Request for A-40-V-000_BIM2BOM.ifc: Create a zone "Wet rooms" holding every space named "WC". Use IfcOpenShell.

First a look at what the model holds.

```python
import ifcopenshell

model = ifcopenshell.open("A-40-V-000_BIM2BOM.ifc")
print(model.schema)
seen = {}
for space in model.by_type("IfcSpace"):
    seen[space.LongName] = seen.get(space.LongName, 0) + 1
for name, count in sorted(seen.items(), key=str):
    print(count, "x", name)
print("zones:", [z.Name for z in model.by_type("IfcZone")][:20])
```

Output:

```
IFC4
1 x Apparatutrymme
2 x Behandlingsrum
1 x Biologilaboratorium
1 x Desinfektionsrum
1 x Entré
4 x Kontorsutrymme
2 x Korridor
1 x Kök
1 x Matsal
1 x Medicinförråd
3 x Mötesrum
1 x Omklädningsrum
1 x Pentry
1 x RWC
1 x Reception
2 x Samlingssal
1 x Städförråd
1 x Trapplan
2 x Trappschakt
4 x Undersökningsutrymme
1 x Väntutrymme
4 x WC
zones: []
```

```python
import ifcopenshell
import ifcopenshell.api.group
import ifcopenshell.api.root

model = ifcopenshell.open("A-40-V-000_BIM2BOM.ifc")

names = {"WC"}
spaces = [s for s in model.by_type("IfcSpace") if s.LongName in names]

zone = ifcopenshell.api.root.create_entity(model, ifc_class="IfcZone", name="Wet rooms")
ifcopenshell.api.group.assign_group(model, products=spaces, group=zone)
print(len(spaces), "spaces in", zone.Name)

model.write("A-40-V-000_BIM2BOM-out.ifc")
```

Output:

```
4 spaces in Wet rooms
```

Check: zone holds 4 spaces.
